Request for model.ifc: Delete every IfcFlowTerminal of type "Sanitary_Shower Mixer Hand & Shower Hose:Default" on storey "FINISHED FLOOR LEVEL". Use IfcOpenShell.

First a look at what the model holds.

```python
import ifcopenshell
import ifcopenshell.util.element

model = ifcopenshell.open("model.ifc")
print(model.schema)
storey = next(s for s in model.by_type("IfcBuildingStorey") if s.Name == "FINISHED FLOOR LEVEL")
terminals = [e for e in ifcopenshell.util.element.get_decomposition(storey) if e.is_a("IfcFlowTerminal")]
seen = {}
for e in terminals:
    element_type = ifcopenshell.util.element.get_type(e)
    name = element_type.Name if element_type not in (None, e) else None
    seen[name] = seen.get(name, 0) + 1
for name, count in sorted(seen.items(), key=str):
    print(count, "x", name)
```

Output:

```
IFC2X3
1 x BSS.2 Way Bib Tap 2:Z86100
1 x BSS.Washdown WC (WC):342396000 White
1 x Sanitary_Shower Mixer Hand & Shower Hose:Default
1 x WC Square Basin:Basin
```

```python
import ifcopenshell
import ifcopenshell.api.root
import ifcopenshell.util.element

model = ifcopenshell.open("model.ifc")

storey = next(s for s in model.by_type("IfcBuildingStorey") if s.Name == "FINISHED FLOOR LEVEL")
terminals = [e for e in ifcopenshell.util.element.get_decomposition(storey) if e.is_a("IfcFlowTerminal")]
targets = [e for e in terminals if (t := ifcopenshell.util.element.get_type(e)) not in (None, e) and t.Name == "Sanitary_Shower Mixer Hand & Shower Hose:Default"]

for e in targets:
    ifcopenshell.api.root.remove_product(model, product=e)
print(len(targets), "removed")

model.write("model_v2.ifc")
```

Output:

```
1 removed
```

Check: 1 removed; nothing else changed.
